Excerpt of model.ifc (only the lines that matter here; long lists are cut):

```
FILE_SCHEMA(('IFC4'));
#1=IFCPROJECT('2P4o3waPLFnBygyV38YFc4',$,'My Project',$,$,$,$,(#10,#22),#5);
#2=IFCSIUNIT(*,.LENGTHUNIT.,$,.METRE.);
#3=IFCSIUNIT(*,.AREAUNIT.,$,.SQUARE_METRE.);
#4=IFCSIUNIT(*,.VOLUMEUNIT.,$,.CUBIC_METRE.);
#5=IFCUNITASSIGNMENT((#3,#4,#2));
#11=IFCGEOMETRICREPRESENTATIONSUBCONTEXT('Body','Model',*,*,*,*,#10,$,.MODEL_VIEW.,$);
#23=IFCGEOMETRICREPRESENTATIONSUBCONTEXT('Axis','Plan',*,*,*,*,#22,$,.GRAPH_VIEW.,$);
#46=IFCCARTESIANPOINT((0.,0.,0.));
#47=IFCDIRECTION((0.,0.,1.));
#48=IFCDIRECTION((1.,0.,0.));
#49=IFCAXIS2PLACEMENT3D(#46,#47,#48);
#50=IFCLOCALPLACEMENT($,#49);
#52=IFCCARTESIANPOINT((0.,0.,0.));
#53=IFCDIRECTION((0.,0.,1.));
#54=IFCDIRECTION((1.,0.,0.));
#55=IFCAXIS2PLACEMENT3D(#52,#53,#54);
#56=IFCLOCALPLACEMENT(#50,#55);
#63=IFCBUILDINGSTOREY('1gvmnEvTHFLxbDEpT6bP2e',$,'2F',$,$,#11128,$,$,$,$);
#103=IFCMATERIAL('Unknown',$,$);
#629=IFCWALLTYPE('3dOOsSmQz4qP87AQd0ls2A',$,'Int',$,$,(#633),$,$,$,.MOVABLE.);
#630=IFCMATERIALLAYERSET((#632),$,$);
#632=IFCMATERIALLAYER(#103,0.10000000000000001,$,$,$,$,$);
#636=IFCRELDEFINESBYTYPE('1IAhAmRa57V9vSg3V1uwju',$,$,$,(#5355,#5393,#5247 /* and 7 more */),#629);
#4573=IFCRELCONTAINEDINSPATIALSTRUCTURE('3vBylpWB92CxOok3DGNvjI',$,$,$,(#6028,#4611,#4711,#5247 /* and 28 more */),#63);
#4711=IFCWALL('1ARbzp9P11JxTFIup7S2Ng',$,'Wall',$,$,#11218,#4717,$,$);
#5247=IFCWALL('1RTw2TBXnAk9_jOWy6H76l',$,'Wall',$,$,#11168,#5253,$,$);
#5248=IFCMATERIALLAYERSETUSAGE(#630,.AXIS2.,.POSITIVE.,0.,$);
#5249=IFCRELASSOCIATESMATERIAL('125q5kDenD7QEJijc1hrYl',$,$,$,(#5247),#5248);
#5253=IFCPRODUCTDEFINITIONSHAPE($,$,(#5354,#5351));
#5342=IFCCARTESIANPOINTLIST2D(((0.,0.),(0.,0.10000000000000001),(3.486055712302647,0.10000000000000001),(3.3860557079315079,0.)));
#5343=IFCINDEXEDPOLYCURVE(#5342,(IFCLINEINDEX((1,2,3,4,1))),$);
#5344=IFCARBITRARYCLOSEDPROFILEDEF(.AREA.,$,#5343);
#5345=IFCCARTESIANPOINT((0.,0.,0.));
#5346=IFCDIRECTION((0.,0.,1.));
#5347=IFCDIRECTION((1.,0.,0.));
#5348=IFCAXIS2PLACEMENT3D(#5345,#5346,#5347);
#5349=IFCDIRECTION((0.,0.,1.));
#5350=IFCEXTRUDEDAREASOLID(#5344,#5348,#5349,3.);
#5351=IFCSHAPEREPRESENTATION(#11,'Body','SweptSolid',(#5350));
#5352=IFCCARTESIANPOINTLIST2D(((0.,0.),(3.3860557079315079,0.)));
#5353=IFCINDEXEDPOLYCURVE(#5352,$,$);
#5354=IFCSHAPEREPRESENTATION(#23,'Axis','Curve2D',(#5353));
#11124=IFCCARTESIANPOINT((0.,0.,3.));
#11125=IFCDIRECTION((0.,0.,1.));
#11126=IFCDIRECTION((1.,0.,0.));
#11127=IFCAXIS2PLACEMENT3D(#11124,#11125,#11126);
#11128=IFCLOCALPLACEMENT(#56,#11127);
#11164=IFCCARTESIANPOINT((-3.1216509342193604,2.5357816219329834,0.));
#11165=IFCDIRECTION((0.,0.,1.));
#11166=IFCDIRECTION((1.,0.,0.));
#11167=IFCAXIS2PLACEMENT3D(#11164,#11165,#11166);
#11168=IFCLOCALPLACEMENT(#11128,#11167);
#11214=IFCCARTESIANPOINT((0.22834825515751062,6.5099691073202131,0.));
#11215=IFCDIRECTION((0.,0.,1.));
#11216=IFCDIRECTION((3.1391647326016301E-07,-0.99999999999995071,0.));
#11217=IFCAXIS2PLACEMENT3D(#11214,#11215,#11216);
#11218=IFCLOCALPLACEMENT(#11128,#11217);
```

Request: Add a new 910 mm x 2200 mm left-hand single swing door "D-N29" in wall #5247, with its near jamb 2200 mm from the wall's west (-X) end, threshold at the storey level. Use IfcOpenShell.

```python
import numpy as np
import ifcopenshell
import ifcopenshell.api.feature
import ifcopenshell.api.geometry
import ifcopenshell.api.root
import ifcopenshell.api.spatial
import ifcopenshell.geom
import ifcopenshell.util.element
import ifcopenshell.util.placement
import ifcopenshell.util.representation
import ifcopenshell.util.shape
import ifcopenshell.util.unit

model = ifcopenshell.open("model.ifc")
unit_scale = ifcopenshell.util.unit.calculate_unit_scale(model)
settings = ifcopenshell.geom.settings()


def volume(element):
    """Net volume in cubic metres, openings subtracted."""
    shape = ifcopenshell.geom.create_shape(settings, element)
    return ifcopenshell.util.shape.get_volume(shape.geometry)


wall = model.by_guid("1RTw2TBXnAk9_jOWy6H76l")
storey = ifcopenshell.util.element.get_container(wall, ifc_class="IfcBuildingStorey")
context = ifcopenshell.util.representation.get_context(model, "Model", "Body", "MODEL_VIEW")
before = volume(wall)

width, height, from_end, sill = 0.91, 2.2, 2.2, 0.0  # metres

# The wall runs along its own X axis, and the end named is its -X end.
wall_shape = ifcopenshell.geom.create_shape(settings, wall)
x, y, z = ifcopenshell.util.shape.get_vertices(wall_shape.geometry).T
start = x.min() + from_end
face, thickness = float(y.min()), float(y.max() - y.min())
wall_matrix = ifcopenshell.util.placement.get_local_placement(wall.ObjectPlacement)
level = ifcopenshell.util.placement.get_local_placement(storey.ObjectPlacement)[2, 3]


def in_wall(x, y):
    """Placement at x, y metres in the wall's axes, at sill height."""
    matrix = wall_matrix.copy()
    matrix[:, 3] = wall_matrix @ np.array([x / unit_scale, y / unit_scale, 0.0, 1.0])
    matrix[2, 3] = level + sill / unit_scale
    return matrix


# Opening: a box that overshoots both wall faces by 50 mm.
opening = ifcopenshell.api.root.create_entity(model, ifc_class="IfcOpeningElement", predefined_type="OPENING")
box = ifcopenshell.api.geometry.add_wall_representation(
    model, context=context, length=width, height=height, thickness=thickness + 0.1
)
ifcopenshell.api.geometry.assign_representation(model, product=opening, representation=box)
ifcopenshell.api.geometry.edit_object_placement(model, product=opening, matrix=in_wall(start, face - 0.05), is_si=False)
ifcopenshell.api.feature.add_feature(model, feature=opening, element=wall)

door = ifcopenshell.api.root.create_entity(model, ifc_class="IfcDoor", name="D-N29", predefined_type="DOOR")
door.OverallWidth, door.OverallHeight = width / unit_scale, height / unit_scale
door.OperationType = "SINGLE_SWING_LEFT"
body = ifcopenshell.api.geometry.add_door_representation(
    model,
    context=context,
    overall_width=door.OverallWidth,
    overall_height=door.OverallHeight,
    operation_type="SINGLE_SWING_LEFT",
    lining_properties={"LiningDepth": thickness / unit_scale, "ThresholdDepth": thickness / unit_scale},
)
ifcopenshell.api.geometry.assign_representation(model, product=door, representation=body)
ifcopenshell.api.spatial.assign_container(model, products=[door], relating_structure=storey)
ifcopenshell.api.feature.add_filling(model, opening=opening, element=door)

# The lining spans the wall, so the door starts at the wall face.
ifcopenshell.api.geometry.edit_object_placement(model, product=door, matrix=in_wall(start, face), is_si=False)

after = volume(wall)

print(f"wall volume {before:.3f} -> {after:.3f} m3")

model.write("model_v2.ifc")
```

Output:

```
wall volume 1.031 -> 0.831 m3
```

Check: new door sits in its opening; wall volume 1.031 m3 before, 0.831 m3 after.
